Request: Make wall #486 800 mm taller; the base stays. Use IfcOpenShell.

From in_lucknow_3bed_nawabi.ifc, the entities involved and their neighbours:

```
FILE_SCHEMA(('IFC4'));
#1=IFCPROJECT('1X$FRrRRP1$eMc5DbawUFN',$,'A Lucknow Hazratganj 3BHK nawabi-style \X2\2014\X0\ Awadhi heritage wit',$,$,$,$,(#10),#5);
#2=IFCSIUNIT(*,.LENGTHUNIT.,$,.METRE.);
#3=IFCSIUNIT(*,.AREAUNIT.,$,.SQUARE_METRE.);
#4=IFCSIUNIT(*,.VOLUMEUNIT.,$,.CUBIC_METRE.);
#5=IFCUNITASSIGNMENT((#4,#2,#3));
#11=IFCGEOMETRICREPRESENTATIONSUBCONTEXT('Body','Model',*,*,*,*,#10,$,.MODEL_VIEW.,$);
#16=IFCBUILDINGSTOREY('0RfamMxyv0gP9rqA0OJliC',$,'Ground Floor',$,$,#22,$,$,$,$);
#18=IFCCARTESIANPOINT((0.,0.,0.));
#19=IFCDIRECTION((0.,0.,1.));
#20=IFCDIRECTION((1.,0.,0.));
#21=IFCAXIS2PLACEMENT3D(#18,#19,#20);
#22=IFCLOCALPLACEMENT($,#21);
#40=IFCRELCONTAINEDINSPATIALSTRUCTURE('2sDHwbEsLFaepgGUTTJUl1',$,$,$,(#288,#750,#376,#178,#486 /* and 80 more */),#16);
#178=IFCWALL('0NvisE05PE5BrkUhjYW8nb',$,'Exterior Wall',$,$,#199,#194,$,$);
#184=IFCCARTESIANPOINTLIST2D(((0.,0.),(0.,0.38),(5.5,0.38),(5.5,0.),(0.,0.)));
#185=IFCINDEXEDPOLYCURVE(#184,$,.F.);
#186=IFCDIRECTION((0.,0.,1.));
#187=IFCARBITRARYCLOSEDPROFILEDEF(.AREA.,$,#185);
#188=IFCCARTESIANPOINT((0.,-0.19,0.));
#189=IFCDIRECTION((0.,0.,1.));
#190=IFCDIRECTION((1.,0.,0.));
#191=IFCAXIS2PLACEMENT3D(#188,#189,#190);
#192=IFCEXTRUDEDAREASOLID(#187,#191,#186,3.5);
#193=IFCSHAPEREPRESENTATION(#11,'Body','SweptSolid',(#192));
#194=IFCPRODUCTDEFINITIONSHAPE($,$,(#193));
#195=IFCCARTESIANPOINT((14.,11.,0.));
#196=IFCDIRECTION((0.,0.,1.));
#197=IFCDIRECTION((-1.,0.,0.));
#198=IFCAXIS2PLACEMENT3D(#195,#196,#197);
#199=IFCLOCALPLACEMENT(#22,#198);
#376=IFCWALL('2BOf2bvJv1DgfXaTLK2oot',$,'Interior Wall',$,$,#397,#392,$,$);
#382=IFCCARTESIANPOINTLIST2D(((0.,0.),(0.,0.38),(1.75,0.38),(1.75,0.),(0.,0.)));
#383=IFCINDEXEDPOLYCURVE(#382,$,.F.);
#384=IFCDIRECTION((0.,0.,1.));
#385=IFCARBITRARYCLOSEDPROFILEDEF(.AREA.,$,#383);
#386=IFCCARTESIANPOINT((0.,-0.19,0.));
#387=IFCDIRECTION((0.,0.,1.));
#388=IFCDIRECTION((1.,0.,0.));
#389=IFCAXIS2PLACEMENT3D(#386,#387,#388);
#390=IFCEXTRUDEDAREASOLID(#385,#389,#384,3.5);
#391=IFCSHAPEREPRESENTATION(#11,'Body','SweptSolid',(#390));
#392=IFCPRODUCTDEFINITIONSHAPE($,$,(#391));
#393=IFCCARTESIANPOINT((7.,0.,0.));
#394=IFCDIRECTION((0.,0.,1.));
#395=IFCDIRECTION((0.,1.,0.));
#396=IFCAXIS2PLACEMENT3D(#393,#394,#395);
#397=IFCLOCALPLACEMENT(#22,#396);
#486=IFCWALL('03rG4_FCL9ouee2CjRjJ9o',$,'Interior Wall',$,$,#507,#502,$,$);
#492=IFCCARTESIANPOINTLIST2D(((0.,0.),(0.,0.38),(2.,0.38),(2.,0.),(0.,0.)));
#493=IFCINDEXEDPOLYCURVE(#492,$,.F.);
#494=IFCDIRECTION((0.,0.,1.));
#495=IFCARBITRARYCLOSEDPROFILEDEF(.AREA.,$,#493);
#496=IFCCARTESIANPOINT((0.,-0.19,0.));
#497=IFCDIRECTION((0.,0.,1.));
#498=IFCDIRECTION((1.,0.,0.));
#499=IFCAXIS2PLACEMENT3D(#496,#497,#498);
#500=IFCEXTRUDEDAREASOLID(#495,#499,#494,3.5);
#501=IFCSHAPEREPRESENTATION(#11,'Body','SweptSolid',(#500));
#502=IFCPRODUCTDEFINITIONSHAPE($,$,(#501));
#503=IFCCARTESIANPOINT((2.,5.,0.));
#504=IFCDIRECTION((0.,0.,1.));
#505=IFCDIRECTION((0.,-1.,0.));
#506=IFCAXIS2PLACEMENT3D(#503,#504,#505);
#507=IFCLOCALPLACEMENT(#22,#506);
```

```python
import ifcopenshell
import ifcopenshell.geom
import ifcopenshell.util.representation
import ifcopenshell.util.shape

model = ifcopenshell.open("in_lucknow_3bed_nawabi.ifc")
settings = ifcopenshell.geom.settings()


def volume(element):
    """Net volume in cubic metres, openings subtracted."""
    shape = ifcopenshell.geom.create_shape(settings, element)
    return ifcopenshell.util.shape.get_volume(shape.geometry)


wall = model.by_id(486)
before = volume(wall)

body = ifcopenshell.util.representation.get_representation(wall, "Model", "Body")
solid = body.Items[0]
old_height = solid.Depth
solid.Depth += 0.8
after = volume(wall)

print(f"height {old_height:g} -> {solid.Depth:g}, volume {before:.3f} -> {after:.3f} m3")

model.write("in_lucknow_3bed_nawabi-out.ifc")
```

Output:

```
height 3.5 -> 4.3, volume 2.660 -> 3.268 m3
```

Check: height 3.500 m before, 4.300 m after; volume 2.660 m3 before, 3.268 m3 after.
